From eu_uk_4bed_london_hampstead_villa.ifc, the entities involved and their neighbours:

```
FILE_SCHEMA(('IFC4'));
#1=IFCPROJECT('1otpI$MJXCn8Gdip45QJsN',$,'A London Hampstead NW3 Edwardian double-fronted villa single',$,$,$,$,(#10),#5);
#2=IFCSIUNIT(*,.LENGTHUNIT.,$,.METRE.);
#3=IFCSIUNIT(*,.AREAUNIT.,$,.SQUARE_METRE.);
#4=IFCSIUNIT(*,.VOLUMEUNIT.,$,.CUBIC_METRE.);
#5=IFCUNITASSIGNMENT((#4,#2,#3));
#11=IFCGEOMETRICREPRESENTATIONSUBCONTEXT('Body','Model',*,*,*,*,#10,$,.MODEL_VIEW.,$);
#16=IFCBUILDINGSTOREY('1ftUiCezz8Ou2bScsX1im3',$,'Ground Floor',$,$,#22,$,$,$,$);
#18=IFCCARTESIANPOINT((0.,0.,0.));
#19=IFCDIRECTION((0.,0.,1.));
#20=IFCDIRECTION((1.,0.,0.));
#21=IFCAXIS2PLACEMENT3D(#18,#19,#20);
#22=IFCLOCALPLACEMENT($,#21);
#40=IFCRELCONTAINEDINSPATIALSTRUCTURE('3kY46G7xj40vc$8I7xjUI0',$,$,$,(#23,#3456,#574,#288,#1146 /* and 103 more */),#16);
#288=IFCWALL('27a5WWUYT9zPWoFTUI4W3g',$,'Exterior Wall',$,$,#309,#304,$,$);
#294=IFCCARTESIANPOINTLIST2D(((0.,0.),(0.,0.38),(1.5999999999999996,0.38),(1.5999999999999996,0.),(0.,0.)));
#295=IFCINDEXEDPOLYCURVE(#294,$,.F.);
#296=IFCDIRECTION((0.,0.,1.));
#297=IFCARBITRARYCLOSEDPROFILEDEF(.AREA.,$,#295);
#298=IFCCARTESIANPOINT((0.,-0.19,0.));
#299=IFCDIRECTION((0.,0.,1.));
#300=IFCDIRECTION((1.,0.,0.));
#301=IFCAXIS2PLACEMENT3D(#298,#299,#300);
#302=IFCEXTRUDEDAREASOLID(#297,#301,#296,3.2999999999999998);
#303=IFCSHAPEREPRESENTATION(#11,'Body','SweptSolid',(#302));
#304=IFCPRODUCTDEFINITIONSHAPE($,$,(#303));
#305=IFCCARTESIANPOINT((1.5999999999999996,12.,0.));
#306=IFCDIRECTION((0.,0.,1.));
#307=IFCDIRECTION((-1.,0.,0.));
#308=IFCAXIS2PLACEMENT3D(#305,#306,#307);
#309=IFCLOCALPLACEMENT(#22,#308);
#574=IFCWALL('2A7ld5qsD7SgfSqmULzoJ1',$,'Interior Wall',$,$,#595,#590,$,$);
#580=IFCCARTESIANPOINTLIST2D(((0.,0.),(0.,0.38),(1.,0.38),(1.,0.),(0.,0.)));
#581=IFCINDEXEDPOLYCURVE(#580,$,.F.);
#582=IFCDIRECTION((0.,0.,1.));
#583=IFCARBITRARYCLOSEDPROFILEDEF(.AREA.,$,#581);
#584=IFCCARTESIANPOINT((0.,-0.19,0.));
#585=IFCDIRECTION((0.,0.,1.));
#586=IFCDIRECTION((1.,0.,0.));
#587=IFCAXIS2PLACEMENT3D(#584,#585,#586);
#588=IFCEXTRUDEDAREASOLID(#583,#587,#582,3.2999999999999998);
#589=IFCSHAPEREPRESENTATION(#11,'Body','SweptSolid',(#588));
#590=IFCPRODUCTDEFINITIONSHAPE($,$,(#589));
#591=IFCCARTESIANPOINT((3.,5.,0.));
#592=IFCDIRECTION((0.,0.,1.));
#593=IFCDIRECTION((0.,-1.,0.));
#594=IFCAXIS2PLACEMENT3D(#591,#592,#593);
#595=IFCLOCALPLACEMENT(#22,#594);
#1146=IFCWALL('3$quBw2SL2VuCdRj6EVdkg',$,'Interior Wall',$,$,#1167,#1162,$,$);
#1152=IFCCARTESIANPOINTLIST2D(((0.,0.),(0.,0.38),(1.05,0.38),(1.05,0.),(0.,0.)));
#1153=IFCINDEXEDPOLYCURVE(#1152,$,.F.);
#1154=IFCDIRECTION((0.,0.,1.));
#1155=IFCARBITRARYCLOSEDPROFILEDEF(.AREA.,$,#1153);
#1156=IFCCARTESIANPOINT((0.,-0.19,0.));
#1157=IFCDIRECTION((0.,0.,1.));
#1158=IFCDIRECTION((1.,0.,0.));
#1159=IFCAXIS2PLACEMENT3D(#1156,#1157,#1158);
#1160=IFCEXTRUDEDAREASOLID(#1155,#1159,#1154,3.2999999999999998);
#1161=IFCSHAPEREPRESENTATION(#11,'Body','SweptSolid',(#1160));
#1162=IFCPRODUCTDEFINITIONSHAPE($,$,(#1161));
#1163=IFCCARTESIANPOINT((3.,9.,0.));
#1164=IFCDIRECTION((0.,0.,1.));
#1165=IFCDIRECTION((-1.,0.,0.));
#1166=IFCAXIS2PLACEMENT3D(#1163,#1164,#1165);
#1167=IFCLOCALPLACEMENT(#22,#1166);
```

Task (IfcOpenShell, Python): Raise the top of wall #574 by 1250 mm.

```python
import ifcopenshell
import ifcopenshell.geom
import ifcopenshell.util.representation
import ifcopenshell.util.shape

model = ifcopenshell.open("eu_uk_4bed_london_hampstead_villa.ifc")
settings = ifcopenshell.geom.settings()


def volume(element):
    """Net volume in cubic metres, openings subtracted."""
    shape = ifcopenshell.geom.create_shape(settings, element)
    return ifcopenshell.util.shape.get_volume(shape.geometry)


wall = model.by_id(574)
before = volume(wall)

body = ifcopenshell.util.representation.get_representation(wall, "Model", "Body")
solid = body.Items[0]
old_height = solid.Depth
solid.Depth += 1.25
after = volume(wall)

print(f"height {old_height:g} -> {solid.Depth:g}, volume {before:.3f} -> {after:.3f} m3")

model.write("eu_uk_4bed_london_hampstead_villa-out.ifc")
```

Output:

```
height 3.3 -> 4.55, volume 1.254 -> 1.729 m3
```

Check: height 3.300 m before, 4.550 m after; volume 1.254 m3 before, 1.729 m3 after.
